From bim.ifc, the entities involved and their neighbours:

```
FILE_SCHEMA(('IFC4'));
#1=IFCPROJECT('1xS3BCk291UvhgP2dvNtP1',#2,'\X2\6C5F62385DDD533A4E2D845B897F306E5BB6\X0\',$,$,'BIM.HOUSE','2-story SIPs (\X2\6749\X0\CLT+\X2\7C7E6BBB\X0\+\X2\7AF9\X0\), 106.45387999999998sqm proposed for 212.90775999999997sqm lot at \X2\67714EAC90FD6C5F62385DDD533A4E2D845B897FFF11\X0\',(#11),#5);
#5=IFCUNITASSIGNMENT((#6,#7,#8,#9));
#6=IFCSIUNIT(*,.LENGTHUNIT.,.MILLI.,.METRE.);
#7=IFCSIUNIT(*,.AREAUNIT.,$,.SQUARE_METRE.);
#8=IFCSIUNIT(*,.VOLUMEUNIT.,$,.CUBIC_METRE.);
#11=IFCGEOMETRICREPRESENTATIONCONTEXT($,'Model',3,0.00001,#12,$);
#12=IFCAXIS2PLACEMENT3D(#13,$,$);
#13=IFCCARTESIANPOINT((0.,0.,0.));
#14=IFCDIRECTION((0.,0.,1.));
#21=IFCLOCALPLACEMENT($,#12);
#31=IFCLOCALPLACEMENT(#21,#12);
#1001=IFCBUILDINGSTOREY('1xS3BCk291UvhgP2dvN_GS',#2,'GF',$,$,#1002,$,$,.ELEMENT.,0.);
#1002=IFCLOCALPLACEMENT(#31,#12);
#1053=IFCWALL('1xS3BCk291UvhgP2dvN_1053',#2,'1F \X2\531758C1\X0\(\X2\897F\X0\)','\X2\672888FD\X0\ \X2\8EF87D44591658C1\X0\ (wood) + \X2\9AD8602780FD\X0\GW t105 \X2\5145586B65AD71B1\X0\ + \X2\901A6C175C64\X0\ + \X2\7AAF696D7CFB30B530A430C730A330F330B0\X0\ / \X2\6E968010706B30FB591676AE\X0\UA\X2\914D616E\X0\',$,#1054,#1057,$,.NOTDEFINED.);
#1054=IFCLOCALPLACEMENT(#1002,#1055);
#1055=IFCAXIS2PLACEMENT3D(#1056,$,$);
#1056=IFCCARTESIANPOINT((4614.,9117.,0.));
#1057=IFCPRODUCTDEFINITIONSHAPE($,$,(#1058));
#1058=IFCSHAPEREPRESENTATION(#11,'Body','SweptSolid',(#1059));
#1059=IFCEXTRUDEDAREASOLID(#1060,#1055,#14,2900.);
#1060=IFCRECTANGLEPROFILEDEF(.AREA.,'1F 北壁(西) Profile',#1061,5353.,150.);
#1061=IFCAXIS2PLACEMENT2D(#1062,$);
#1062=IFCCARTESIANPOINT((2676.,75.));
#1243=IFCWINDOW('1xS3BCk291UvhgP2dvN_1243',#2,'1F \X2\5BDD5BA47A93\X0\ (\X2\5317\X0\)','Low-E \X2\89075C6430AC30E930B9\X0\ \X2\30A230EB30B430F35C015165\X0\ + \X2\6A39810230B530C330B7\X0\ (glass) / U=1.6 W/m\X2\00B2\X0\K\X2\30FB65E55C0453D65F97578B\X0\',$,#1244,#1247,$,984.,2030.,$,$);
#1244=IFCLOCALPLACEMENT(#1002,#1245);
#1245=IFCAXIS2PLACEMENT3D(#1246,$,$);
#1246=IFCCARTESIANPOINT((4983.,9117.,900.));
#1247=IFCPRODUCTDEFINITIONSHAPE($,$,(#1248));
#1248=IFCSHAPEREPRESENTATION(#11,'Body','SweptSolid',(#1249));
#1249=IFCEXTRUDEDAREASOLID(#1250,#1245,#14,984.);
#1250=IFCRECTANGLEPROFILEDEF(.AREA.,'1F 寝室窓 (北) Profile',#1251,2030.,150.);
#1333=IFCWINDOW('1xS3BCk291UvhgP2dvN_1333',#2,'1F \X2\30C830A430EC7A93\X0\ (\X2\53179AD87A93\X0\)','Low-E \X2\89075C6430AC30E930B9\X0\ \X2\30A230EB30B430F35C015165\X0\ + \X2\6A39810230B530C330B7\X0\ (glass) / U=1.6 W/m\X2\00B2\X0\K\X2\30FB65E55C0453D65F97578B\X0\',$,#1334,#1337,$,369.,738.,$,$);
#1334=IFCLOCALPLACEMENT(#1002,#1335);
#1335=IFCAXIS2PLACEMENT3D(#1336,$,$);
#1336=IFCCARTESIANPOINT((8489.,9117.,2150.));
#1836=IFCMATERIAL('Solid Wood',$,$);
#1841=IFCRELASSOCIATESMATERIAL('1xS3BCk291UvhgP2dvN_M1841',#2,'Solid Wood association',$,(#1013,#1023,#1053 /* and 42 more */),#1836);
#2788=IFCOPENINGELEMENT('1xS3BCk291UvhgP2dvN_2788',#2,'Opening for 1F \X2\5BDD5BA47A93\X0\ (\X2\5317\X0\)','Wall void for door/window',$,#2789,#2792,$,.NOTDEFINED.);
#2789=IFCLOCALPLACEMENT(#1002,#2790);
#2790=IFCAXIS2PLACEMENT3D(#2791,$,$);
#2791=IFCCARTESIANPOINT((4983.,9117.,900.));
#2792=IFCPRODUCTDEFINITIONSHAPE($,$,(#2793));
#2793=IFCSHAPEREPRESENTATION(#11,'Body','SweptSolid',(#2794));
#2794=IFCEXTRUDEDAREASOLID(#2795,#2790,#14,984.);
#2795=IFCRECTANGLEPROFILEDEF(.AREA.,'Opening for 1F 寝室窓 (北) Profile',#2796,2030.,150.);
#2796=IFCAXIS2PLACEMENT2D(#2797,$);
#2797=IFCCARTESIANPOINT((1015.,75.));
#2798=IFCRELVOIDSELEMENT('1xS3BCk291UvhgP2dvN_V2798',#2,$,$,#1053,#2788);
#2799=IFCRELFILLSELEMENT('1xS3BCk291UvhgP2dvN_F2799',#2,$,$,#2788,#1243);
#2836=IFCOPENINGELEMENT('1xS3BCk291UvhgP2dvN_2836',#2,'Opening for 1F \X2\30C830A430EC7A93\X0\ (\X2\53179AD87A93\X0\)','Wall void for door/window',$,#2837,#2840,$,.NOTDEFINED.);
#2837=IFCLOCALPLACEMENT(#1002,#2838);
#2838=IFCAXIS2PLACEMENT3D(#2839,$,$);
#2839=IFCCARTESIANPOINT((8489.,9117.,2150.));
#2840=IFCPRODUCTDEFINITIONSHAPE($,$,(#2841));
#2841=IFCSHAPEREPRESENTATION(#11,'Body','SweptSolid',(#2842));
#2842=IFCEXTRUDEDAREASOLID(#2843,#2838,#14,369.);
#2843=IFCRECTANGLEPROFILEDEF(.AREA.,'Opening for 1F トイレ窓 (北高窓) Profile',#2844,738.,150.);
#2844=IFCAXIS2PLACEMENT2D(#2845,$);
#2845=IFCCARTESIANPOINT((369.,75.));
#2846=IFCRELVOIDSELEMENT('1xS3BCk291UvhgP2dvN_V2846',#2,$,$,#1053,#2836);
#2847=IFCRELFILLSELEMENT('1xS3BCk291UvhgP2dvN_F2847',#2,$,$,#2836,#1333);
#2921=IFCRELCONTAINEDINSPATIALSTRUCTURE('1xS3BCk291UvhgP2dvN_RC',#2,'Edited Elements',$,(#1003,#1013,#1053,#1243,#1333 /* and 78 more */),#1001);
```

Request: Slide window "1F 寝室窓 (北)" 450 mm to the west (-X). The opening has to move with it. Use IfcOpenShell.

```python
import ifcopenshell
import ifcopenshell.api.geometry
import ifcopenshell.util.placement
import ifcopenshell.util.unit

model = ifcopenshell.open("bim.ifc")
unit_scale = ifcopenshell.util.unit.calculate_unit_scale(model)

window = model.by_guid("1xS3BCk291UvhgP2dvN_1243")
opening = window.FillsVoids[0].RelatingOpeningElement
wall = opening.VoidsElements[0].RelatingBuildingElement

wall_matrix = ifcopenshell.util.placement.get_local_placement(wall.ObjectPlacement)
shift = wall_matrix[:3, 0] * -0.45 / unit_scale
before = ifcopenshell.util.placement.get_local_placement(window.ObjectPlacement)[:3, 3].copy()

# The window is not placed relative to its opening, so move both.
for product in (opening, window):
    matrix = ifcopenshell.util.placement.get_local_placement(product.ObjectPlacement)
    matrix[:3, 3] += shift
    ifcopenshell.api.geometry.edit_object_placement(model, product=product, matrix=matrix, is_si=False)

after = ifcopenshell.util.placement.get_local_placement(window.ObjectPlacement)[:3, 3]
print("window moved by", (after - before).round(3) + 0.0)

model.write("bim-out.ifc")
```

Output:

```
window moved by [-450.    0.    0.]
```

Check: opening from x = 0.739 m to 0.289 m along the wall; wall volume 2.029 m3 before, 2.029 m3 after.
